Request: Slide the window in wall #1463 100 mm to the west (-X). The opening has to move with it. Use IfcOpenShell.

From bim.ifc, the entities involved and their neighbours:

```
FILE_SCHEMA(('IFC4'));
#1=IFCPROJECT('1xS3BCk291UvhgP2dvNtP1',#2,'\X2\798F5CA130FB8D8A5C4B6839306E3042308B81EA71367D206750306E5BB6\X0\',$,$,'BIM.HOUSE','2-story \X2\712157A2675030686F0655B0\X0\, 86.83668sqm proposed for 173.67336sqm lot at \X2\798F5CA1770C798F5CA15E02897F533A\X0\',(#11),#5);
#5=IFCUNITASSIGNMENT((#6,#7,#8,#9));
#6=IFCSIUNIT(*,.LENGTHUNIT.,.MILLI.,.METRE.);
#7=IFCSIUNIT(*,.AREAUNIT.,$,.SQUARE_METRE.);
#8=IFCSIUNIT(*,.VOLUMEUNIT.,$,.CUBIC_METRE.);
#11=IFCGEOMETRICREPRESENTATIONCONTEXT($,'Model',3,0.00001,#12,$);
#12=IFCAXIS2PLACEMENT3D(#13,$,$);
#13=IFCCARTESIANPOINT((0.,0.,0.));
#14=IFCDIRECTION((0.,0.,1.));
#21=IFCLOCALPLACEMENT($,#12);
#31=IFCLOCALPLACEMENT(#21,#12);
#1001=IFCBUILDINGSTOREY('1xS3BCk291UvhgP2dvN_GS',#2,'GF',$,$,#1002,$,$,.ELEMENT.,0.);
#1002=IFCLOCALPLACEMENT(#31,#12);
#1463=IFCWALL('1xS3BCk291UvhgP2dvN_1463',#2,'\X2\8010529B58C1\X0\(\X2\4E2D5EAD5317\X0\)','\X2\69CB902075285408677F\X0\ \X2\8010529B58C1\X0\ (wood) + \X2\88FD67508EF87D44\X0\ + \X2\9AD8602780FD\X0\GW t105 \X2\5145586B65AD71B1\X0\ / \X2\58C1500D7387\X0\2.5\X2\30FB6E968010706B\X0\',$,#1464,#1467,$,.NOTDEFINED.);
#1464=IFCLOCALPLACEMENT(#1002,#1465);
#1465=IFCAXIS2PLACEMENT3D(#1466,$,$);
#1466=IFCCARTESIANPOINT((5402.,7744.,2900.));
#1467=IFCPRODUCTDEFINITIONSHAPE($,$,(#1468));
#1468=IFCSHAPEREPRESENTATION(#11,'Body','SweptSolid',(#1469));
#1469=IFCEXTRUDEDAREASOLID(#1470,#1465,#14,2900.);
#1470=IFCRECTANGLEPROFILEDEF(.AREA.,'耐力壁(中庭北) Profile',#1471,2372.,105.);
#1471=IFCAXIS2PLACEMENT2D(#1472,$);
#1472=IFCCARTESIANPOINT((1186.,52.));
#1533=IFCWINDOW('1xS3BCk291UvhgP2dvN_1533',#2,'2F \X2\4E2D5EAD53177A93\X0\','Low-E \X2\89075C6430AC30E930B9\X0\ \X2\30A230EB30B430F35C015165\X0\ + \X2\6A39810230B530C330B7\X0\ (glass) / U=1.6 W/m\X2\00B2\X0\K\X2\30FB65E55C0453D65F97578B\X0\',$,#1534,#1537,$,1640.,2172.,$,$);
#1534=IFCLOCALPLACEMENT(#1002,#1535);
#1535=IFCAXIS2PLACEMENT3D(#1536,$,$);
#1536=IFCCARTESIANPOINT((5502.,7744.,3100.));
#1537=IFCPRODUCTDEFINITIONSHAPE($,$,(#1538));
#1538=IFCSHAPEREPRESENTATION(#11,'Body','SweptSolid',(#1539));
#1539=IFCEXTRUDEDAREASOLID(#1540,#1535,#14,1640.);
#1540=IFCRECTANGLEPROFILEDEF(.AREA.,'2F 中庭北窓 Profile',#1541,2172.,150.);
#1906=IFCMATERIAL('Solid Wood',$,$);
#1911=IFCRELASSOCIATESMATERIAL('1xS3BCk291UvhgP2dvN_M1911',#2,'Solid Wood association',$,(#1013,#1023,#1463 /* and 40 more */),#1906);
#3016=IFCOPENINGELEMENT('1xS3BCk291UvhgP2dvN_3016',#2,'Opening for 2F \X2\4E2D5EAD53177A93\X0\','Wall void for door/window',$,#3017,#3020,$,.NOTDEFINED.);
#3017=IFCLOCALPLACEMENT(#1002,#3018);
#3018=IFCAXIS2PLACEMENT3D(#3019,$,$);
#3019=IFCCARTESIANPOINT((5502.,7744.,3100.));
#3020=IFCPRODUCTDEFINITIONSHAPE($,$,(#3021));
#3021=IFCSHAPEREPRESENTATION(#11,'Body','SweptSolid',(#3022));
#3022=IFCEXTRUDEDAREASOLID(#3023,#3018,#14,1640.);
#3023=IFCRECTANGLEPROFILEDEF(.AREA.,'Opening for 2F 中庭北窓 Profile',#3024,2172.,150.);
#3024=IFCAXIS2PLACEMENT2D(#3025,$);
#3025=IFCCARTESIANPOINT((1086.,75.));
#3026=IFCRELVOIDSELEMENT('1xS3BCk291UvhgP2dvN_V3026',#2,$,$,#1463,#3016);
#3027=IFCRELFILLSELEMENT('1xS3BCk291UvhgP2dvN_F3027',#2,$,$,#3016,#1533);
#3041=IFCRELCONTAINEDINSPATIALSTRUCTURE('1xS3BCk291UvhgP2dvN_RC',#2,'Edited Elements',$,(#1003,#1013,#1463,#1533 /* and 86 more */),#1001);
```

```python
import ifcopenshell
import ifcopenshell.api.geometry
import ifcopenshell.util.placement
import ifcopenshell.util.unit

model = ifcopenshell.open("bim.ifc")
unit_scale = ifcopenshell.util.unit.calculate_unit_scale(model)

window = model.by_id(1533)
opening = window.FillsVoids[0].RelatingOpeningElement
wall = opening.VoidsElements[0].RelatingBuildingElement

wall_matrix = ifcopenshell.util.placement.get_local_placement(wall.ObjectPlacement)
shift = wall_matrix[:3, 0] * -0.1 / unit_scale
before = ifcopenshell.util.placement.get_local_placement(window.ObjectPlacement)[:3, 3].copy()

# The window is not placed relative to its opening, so move both.
for product in (opening, window):
    matrix = ifcopenshell.util.placement.get_local_placement(product.ObjectPlacement)
    matrix[:3, 3] += shift
    ifcopenshell.api.geometry.edit_object_placement(model, product=product, matrix=matrix, is_si=False)

after = ifcopenshell.util.placement.get_local_placement(window.ObjectPlacement)[:3, 3]
print("window moved by", (after - before).round(3) + 0.0)

model.write("bim_updated.ifc")
```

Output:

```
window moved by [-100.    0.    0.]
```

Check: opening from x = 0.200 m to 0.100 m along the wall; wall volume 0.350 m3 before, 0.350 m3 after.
